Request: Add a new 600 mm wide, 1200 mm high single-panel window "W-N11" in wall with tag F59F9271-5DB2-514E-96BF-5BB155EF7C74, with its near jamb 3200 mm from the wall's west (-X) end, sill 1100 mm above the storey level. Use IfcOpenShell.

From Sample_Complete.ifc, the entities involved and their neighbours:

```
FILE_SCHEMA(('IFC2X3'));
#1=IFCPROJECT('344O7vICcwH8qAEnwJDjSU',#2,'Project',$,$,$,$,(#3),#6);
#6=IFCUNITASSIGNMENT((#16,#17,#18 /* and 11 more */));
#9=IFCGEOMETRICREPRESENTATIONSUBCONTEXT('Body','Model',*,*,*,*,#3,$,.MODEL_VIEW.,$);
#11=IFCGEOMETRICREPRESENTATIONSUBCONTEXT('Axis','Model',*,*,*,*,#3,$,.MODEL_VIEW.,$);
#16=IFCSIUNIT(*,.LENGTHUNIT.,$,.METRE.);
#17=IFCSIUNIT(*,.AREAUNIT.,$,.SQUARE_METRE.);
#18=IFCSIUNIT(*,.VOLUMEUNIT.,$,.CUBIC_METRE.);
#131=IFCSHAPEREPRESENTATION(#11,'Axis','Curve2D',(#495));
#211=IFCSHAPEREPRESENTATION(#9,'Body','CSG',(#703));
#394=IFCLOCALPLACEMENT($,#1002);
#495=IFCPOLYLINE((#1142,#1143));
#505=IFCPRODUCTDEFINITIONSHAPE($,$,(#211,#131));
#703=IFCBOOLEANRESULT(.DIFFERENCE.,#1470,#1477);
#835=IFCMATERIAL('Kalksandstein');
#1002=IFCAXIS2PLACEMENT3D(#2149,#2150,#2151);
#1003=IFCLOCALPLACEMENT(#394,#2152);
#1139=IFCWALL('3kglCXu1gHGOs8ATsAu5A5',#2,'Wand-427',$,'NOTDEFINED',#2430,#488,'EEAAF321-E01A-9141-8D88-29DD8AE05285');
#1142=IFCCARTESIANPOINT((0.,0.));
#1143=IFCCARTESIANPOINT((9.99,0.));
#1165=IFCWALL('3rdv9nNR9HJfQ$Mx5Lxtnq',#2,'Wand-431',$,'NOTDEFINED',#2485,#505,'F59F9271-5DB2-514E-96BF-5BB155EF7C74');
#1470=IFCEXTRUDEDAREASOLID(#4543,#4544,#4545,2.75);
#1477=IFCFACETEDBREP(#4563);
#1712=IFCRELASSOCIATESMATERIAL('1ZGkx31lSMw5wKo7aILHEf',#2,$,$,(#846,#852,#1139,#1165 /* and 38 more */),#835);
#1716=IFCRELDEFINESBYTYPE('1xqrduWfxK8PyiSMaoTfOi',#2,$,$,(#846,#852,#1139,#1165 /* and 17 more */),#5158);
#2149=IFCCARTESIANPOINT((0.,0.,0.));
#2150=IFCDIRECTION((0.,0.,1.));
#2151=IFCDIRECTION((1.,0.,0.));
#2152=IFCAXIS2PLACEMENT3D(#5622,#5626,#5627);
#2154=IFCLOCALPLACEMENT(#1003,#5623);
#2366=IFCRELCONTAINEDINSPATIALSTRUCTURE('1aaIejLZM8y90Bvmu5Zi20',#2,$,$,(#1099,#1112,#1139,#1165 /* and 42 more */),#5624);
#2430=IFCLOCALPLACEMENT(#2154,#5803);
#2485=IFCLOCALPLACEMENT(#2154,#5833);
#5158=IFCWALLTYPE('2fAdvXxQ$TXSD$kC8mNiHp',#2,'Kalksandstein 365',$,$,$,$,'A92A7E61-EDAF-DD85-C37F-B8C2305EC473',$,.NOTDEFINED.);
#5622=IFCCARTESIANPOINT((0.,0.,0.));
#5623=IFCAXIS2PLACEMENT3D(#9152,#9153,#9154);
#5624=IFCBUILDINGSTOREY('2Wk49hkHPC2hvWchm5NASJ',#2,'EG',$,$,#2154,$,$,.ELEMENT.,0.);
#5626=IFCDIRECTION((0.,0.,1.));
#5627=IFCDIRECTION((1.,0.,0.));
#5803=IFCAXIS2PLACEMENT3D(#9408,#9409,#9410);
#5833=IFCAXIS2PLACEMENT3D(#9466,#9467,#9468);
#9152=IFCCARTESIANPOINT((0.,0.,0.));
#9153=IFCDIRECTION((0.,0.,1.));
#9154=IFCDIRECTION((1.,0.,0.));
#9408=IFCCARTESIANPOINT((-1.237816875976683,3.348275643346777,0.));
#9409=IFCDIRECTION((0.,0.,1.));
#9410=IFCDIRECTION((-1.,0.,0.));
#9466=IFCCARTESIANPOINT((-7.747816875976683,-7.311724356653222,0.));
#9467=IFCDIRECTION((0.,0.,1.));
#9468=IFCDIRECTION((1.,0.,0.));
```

```python
import numpy as np
import ifcopenshell
import ifcopenshell.api.feature
import ifcopenshell.api.geometry
import ifcopenshell.api.root
import ifcopenshell.api.spatial
import ifcopenshell.api.type
import ifcopenshell.geom
import ifcopenshell.util.element
import ifcopenshell.util.placement
import ifcopenshell.util.representation
import ifcopenshell.util.shape
import ifcopenshell.util.unit

model = ifcopenshell.open("Sample_Complete.ifc")
unit_scale = ifcopenshell.util.unit.calculate_unit_scale(model)
settings = ifcopenshell.geom.settings()


def volume(element):
    """Net volume in cubic metres, openings subtracted."""
    shape = ifcopenshell.geom.create_shape(settings, element)
    return ifcopenshell.util.shape.get_volume(shape.geometry)


wall = model.by_guid("3rdv9nNR9HJfQ$Mx5Lxtnq")
storey = ifcopenshell.util.element.get_container(wall, ifc_class="IfcBuildingStorey")
context = ifcopenshell.util.representation.get_context(model, "Model", "Body", "MODEL_VIEW")
before = volume(wall)

width, height, from_end, sill = 0.6, 1.2, 3.2, 1.1  # metres

# The wall runs along its own X axis, and the end named is its -X end.
wall_shape = ifcopenshell.geom.create_shape(settings, wall)
x, y, z = ifcopenshell.util.shape.get_vertices(wall_shape.geometry).T
start = x.min() + from_end
face, thickness = float(y.min()), float(y.max() - y.min())
wall_matrix = ifcopenshell.util.placement.get_local_placement(wall.ObjectPlacement)
level = ifcopenshell.util.placement.get_local_placement(storey.ObjectPlacement)[2, 3]


def in_wall(x, y):
    """Placement at x, y metres in the wall's axes, at sill height."""
    matrix = wall_matrix.copy()
    matrix[:, 3] = wall_matrix @ np.array([x / unit_scale, y / unit_scale, 0.0, 1.0])
    matrix[2, 3] = level + sill / unit_scale
    return matrix


# Opening: a box that overshoots both wall faces by 50 mm.
opening = ifcopenshell.api.root.create_entity(model, ifc_class="IfcOpeningElement")
box = ifcopenshell.api.geometry.add_wall_representation(
    model, context=context, length=width, height=height, thickness=thickness + 0.1
)
ifcopenshell.api.geometry.assign_representation(model, product=opening, representation=box)
ifcopenshell.api.geometry.edit_object_placement(model, product=opening, matrix=in_wall(start, face - 0.05), is_si=False)
ifcopenshell.api.feature.add_feature(model, feature=opening, element=wall)

window = ifcopenshell.api.root.create_entity(model, ifc_class="IfcWindow", name="W-N11")
window.OverallWidth, window.OverallHeight = width / unit_scale, height / unit_scale
body = ifcopenshell.api.geometry.add_window_representation(
    model,
    context=context,
    overall_width=window.OverallWidth,
    overall_height=window.OverallHeight,
    partition_type="SINGLE_PANEL",
)
ifcopenshell.api.geometry.assign_representation(model, product=window, representation=body)
ifcopenshell.api.spatial.assign_container(model, products=[window], relating_structure=storey)
fills = ifcopenshell.api.feature.add_filling(model, opening=opening, element=window)
fills.OwnerHistory = window.OwnerHistory  # required in IFC2X3

# IFC2X3 keeps the operation on the window style.
style = ifcopenshell.api.root.create_entity(model, ifc_class="IfcWindowStyle", name="W-N11")
style.OperationType, style.ConstructionType = "SINGLE_PANEL", "NOTDEFINED"
style.ParameterTakesPrecedence = style.Sizeable = False
ifcopenshell.api.type.assign_type(model, related_objects=[window], relating_type=style)

# Centre the window in the wall's thickness.
ifcopenshell.api.geometry.edit_object_placement(model, product=window, matrix=in_wall(start, face), is_si=False)
window_shape = ifcopenshell.geom.create_shape(settings, window)
depth = ifcopenshell.util.shape.get_vertices(window_shape.geometry)[:, 1]
offset = face + thickness / 2 - (depth.min() + depth.max()) / 2
ifcopenshell.api.geometry.edit_object_placement(model, product=window, matrix=in_wall(start, offset), is_si=False)

after = volume(wall)

print(f"wall volume {before:.3f} -> {after:.3f} m3")

model.write("Sample_Complete_rev.ifc")
```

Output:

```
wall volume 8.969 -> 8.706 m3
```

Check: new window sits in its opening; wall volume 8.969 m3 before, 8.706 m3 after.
